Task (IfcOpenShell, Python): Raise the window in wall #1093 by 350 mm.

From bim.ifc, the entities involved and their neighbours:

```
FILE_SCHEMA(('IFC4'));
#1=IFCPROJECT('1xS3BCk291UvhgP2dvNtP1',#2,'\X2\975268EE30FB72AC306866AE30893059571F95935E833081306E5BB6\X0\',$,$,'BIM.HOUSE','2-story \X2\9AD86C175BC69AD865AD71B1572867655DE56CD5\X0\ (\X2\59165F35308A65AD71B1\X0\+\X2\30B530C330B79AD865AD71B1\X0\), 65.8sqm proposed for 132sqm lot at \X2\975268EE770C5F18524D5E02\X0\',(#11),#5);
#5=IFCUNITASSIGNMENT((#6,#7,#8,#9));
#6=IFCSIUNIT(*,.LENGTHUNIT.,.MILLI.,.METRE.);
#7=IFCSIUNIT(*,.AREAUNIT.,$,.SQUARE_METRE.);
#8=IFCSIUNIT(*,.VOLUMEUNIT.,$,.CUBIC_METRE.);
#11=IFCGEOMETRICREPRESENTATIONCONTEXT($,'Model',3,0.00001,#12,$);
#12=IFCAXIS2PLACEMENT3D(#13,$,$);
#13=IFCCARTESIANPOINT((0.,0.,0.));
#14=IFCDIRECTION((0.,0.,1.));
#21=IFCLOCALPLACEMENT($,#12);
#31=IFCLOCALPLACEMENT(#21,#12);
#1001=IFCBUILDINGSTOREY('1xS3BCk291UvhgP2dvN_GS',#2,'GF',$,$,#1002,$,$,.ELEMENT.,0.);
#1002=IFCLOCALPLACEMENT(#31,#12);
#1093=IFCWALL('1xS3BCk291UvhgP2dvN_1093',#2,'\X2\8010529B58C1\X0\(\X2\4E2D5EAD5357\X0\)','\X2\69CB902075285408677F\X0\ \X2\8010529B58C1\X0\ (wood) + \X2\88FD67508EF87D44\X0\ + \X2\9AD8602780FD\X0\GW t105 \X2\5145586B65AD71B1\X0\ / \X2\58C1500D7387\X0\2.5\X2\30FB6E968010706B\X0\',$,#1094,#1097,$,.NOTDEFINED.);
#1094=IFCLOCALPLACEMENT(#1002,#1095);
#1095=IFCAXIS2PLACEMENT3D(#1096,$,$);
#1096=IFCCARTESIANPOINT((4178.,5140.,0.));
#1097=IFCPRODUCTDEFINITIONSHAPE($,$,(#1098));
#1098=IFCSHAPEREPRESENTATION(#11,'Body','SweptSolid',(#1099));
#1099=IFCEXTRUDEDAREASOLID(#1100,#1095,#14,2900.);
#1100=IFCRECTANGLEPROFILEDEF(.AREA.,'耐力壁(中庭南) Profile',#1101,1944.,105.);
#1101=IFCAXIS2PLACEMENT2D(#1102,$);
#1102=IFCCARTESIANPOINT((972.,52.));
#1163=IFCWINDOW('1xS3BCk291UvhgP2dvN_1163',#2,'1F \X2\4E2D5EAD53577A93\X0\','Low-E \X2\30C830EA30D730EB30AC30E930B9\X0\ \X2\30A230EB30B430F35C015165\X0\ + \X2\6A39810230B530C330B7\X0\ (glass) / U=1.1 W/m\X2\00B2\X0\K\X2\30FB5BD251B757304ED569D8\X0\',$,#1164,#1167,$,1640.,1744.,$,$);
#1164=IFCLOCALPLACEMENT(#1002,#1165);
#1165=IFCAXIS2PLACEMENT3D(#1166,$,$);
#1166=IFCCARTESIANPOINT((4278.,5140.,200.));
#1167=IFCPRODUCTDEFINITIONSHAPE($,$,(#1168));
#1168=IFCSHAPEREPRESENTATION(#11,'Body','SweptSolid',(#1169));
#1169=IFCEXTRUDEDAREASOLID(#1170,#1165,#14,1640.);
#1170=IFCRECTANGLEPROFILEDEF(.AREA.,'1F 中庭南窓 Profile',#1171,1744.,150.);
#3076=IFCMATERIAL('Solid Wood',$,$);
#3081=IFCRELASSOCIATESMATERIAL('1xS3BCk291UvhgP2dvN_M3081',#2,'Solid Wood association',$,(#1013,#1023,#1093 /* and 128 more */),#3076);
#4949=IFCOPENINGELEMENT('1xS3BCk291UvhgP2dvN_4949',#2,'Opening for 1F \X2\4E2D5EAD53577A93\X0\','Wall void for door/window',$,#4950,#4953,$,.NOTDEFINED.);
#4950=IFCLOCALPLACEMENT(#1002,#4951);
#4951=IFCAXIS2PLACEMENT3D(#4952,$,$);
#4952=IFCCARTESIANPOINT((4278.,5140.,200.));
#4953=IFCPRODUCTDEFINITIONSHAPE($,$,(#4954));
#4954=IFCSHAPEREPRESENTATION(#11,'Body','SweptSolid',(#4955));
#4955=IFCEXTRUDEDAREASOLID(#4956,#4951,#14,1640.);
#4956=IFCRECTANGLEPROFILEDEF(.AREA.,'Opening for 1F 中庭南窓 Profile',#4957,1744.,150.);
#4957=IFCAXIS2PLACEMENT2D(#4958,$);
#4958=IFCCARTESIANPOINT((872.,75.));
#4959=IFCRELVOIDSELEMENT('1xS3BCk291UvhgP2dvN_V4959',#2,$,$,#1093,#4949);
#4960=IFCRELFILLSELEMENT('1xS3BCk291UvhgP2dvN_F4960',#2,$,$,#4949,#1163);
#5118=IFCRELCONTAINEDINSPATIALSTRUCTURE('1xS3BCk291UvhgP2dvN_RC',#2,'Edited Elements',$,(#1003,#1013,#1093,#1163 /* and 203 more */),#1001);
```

```python
import numpy as np
import ifcopenshell
import ifcopenshell.api.geometry
import ifcopenshell.util.placement
import ifcopenshell.util.unit

model = ifcopenshell.open("bim.ifc")
unit_scale = ifcopenshell.util.unit.calculate_unit_scale(model)

window = model.by_guid("1xS3BCk291UvhgP2dvN_1163")
opening = window.FillsVoids[0].RelatingOpeningElement
dz = 0.35 / unit_scale

shift = np.array([0.0, 0.0, dz])
# The window is not placed relative to its opening, so move both.
for product in (opening, window):
    matrix = ifcopenshell.util.placement.get_local_placement(product.ObjectPlacement)
    matrix[:3, 3] += shift
    ifcopenshell.api.geometry.edit_object_placement(model, product=product, matrix=matrix, is_si=False)

print(f"moved by {dz * unit_scale:+.3f} m")

model.write("bim_edited.ifc")
```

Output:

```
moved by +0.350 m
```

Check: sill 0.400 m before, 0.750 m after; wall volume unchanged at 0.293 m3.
